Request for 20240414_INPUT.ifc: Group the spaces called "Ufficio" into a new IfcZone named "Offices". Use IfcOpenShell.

First a look at what the model holds.

```python
import ifcopenshell

model = ifcopenshell.open("20240414_INPUT.ifc")
print(model.schema)
seen = {}
for space in model.by_type("IfcSpace"):
    seen[space.LongName] = seen.get(space.LongName, 0) + 1
for name, count in sorted(seen.items(), key=str):
    print(count, "x", name)
print("zones:", [z.Name for z in model.by_type("IfcZone")][:20])
```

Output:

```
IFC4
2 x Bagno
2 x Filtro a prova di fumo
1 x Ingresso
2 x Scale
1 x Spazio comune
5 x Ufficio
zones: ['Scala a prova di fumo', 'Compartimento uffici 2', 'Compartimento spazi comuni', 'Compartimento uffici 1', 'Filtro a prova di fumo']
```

```python
import ifcopenshell
import ifcopenshell.api.group
import ifcopenshell.api.root

model = ifcopenshell.open("20240414_INPUT.ifc")

names = {"Ufficio"}
spaces = [s for s in model.by_type("IfcSpace") if s.LongName in names]

zone = ifcopenshell.api.root.create_entity(model, ifc_class="IfcZone", name="Offices")
ifcopenshell.api.group.assign_group(model, products=spaces, group=zone)
print(len(spaces), "spaces in", zone.Name)

model.write("20240414_INPUT_v2.ifc")
```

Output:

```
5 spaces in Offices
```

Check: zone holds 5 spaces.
